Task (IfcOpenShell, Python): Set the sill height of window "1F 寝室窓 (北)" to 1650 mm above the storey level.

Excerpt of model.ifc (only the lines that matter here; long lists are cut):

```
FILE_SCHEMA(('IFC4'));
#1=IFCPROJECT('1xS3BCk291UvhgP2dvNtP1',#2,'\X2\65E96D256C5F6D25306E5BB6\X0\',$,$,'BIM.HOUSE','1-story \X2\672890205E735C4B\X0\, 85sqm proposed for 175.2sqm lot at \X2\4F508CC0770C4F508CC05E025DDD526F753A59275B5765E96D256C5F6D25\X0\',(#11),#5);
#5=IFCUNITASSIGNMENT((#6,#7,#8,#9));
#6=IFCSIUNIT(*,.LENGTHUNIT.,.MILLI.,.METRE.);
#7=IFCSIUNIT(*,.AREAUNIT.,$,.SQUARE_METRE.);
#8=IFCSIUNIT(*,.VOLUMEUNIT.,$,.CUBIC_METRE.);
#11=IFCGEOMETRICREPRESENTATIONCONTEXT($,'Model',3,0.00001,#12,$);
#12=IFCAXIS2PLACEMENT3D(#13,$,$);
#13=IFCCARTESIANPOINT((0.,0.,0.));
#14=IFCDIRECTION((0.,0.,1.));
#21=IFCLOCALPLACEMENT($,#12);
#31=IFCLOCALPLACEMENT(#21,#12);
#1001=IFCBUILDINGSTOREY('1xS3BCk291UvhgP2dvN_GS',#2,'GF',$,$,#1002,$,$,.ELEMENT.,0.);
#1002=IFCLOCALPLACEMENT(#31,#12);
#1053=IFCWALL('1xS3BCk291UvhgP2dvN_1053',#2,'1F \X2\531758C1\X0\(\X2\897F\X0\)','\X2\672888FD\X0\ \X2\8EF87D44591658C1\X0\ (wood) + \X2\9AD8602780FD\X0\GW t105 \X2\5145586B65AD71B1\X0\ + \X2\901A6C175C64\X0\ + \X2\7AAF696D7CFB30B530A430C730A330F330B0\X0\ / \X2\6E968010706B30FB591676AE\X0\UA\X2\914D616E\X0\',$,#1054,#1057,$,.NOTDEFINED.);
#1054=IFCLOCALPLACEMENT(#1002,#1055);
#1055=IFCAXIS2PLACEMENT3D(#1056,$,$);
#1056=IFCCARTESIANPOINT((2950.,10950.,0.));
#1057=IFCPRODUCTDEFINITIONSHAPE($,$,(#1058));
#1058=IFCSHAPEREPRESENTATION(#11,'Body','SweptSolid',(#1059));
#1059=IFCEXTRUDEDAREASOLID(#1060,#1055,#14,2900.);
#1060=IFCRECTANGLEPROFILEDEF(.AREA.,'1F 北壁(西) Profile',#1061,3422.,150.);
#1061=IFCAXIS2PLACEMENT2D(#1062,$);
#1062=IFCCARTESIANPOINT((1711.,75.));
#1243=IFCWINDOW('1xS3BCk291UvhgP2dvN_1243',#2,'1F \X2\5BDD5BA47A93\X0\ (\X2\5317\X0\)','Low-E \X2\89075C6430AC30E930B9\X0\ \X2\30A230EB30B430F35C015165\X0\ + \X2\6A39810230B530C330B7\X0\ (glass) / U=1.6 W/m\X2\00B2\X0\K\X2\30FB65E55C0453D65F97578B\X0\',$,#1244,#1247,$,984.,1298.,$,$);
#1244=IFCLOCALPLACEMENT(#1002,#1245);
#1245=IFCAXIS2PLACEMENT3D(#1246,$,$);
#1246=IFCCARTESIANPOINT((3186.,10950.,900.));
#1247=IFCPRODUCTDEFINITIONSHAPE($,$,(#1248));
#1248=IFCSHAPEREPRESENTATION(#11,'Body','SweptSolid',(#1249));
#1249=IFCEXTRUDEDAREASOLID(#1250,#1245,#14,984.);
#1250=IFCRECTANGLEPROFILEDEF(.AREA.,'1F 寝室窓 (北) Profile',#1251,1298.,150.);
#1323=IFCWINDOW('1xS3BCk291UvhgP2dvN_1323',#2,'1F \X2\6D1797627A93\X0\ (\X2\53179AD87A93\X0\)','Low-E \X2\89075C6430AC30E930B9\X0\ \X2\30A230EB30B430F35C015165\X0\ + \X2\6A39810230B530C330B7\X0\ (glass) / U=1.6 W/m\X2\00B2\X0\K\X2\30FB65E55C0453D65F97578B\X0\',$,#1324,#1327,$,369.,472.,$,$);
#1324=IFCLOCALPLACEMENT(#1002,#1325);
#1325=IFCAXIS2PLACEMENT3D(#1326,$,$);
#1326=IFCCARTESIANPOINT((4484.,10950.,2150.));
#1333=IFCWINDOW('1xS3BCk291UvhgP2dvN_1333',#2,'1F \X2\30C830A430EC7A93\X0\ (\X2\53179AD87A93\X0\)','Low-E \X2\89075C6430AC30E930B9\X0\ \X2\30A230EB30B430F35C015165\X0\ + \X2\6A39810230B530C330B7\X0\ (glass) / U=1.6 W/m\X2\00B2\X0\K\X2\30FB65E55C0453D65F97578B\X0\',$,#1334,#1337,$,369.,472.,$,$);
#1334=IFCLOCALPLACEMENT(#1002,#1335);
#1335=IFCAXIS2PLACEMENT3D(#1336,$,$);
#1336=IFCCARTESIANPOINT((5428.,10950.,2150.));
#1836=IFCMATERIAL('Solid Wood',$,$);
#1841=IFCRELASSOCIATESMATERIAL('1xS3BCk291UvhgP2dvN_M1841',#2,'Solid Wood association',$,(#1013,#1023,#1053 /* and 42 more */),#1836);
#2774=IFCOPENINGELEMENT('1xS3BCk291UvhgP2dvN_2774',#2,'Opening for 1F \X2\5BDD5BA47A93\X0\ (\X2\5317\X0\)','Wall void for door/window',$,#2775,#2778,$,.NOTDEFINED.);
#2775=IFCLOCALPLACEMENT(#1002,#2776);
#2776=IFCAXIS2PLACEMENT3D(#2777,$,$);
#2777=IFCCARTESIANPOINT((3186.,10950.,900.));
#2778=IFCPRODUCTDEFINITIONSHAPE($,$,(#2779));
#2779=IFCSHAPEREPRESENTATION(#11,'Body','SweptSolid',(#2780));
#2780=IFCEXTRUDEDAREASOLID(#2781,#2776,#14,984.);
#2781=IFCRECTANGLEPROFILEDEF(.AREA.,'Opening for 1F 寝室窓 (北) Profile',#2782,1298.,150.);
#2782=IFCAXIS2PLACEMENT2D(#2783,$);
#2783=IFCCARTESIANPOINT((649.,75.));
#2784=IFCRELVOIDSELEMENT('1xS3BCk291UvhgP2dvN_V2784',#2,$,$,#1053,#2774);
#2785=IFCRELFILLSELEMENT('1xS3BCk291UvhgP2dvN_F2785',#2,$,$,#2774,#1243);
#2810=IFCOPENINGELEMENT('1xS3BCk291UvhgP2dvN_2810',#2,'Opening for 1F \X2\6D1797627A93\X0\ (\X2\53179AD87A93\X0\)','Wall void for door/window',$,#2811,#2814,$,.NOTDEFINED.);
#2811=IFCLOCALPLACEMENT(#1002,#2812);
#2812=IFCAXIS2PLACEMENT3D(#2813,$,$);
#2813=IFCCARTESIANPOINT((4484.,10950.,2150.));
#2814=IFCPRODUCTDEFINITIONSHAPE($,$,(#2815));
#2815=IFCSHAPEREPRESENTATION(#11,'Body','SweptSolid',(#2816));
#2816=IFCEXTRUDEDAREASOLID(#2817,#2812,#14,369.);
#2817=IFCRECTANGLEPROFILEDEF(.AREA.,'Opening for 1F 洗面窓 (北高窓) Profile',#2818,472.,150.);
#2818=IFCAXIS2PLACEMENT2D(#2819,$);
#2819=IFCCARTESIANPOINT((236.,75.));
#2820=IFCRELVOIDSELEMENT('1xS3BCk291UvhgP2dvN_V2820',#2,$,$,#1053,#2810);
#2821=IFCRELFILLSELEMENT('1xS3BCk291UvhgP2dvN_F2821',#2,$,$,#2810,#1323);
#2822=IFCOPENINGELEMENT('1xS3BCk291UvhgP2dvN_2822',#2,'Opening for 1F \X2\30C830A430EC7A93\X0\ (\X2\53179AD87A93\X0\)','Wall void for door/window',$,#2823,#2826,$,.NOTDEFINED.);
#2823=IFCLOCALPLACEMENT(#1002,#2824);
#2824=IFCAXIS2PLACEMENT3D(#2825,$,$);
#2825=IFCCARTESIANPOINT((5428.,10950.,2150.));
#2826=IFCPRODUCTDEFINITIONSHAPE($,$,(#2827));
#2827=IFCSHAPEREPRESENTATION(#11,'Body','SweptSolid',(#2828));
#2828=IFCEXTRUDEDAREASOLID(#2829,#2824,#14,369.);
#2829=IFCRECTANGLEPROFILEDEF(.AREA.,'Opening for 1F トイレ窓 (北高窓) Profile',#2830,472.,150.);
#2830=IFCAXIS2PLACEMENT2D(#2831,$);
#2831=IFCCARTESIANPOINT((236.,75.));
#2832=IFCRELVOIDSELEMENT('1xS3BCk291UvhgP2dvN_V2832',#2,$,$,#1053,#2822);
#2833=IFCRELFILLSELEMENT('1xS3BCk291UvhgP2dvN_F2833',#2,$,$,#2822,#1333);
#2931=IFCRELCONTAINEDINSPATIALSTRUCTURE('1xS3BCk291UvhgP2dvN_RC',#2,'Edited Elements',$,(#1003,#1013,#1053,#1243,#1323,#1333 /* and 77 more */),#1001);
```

```python
import numpy as np
import ifcopenshell
import ifcopenshell.api.geometry
import ifcopenshell.geom
import ifcopenshell.util.element
import ifcopenshell.util.placement
import ifcopenshell.util.shape
import ifcopenshell.util.unit

model = ifcopenshell.open("model.ifc")
unit_scale = ifcopenshell.util.unit.calculate_unit_scale(model)

window = model.by_guid("1xS3BCk291UvhgP2dvN_1243")
opening = window.FillsVoids[0].RelatingOpeningElement
storey = ifcopenshell.util.element.get_container(window, ifc_class="IfcBuildingStorey")
level = ifcopenshell.util.placement.get_local_placement(storey.ObjectPlacement)[2, 3]

# The opening's origin need not be at the sill, so measure its lowest point.
shape = ifcopenshell.geom.create_shape(ifcopenshell.geom.settings(), opening)
bottom = ifcopenshell.util.shape.get_shape_bottom_elevation(shape, shape.geometry) / unit_scale
dz = level + 1.65 / unit_scale - bottom

shift = np.array([0.0, 0.0, dz])
# The window is not placed relative to its opening, so move both.
for product in (opening, window):
    matrix = ifcopenshell.util.placement.get_local_placement(product.ObjectPlacement)
    matrix[:3, 3] += shift
    ifcopenshell.api.geometry.edit_object_placement(model, product=product, matrix=matrix, is_si=False)

print(f"moved by {dz * unit_scale:+.3f} m")

model.write("model_updated.ifc")
```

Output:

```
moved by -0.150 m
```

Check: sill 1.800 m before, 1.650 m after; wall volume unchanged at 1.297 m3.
